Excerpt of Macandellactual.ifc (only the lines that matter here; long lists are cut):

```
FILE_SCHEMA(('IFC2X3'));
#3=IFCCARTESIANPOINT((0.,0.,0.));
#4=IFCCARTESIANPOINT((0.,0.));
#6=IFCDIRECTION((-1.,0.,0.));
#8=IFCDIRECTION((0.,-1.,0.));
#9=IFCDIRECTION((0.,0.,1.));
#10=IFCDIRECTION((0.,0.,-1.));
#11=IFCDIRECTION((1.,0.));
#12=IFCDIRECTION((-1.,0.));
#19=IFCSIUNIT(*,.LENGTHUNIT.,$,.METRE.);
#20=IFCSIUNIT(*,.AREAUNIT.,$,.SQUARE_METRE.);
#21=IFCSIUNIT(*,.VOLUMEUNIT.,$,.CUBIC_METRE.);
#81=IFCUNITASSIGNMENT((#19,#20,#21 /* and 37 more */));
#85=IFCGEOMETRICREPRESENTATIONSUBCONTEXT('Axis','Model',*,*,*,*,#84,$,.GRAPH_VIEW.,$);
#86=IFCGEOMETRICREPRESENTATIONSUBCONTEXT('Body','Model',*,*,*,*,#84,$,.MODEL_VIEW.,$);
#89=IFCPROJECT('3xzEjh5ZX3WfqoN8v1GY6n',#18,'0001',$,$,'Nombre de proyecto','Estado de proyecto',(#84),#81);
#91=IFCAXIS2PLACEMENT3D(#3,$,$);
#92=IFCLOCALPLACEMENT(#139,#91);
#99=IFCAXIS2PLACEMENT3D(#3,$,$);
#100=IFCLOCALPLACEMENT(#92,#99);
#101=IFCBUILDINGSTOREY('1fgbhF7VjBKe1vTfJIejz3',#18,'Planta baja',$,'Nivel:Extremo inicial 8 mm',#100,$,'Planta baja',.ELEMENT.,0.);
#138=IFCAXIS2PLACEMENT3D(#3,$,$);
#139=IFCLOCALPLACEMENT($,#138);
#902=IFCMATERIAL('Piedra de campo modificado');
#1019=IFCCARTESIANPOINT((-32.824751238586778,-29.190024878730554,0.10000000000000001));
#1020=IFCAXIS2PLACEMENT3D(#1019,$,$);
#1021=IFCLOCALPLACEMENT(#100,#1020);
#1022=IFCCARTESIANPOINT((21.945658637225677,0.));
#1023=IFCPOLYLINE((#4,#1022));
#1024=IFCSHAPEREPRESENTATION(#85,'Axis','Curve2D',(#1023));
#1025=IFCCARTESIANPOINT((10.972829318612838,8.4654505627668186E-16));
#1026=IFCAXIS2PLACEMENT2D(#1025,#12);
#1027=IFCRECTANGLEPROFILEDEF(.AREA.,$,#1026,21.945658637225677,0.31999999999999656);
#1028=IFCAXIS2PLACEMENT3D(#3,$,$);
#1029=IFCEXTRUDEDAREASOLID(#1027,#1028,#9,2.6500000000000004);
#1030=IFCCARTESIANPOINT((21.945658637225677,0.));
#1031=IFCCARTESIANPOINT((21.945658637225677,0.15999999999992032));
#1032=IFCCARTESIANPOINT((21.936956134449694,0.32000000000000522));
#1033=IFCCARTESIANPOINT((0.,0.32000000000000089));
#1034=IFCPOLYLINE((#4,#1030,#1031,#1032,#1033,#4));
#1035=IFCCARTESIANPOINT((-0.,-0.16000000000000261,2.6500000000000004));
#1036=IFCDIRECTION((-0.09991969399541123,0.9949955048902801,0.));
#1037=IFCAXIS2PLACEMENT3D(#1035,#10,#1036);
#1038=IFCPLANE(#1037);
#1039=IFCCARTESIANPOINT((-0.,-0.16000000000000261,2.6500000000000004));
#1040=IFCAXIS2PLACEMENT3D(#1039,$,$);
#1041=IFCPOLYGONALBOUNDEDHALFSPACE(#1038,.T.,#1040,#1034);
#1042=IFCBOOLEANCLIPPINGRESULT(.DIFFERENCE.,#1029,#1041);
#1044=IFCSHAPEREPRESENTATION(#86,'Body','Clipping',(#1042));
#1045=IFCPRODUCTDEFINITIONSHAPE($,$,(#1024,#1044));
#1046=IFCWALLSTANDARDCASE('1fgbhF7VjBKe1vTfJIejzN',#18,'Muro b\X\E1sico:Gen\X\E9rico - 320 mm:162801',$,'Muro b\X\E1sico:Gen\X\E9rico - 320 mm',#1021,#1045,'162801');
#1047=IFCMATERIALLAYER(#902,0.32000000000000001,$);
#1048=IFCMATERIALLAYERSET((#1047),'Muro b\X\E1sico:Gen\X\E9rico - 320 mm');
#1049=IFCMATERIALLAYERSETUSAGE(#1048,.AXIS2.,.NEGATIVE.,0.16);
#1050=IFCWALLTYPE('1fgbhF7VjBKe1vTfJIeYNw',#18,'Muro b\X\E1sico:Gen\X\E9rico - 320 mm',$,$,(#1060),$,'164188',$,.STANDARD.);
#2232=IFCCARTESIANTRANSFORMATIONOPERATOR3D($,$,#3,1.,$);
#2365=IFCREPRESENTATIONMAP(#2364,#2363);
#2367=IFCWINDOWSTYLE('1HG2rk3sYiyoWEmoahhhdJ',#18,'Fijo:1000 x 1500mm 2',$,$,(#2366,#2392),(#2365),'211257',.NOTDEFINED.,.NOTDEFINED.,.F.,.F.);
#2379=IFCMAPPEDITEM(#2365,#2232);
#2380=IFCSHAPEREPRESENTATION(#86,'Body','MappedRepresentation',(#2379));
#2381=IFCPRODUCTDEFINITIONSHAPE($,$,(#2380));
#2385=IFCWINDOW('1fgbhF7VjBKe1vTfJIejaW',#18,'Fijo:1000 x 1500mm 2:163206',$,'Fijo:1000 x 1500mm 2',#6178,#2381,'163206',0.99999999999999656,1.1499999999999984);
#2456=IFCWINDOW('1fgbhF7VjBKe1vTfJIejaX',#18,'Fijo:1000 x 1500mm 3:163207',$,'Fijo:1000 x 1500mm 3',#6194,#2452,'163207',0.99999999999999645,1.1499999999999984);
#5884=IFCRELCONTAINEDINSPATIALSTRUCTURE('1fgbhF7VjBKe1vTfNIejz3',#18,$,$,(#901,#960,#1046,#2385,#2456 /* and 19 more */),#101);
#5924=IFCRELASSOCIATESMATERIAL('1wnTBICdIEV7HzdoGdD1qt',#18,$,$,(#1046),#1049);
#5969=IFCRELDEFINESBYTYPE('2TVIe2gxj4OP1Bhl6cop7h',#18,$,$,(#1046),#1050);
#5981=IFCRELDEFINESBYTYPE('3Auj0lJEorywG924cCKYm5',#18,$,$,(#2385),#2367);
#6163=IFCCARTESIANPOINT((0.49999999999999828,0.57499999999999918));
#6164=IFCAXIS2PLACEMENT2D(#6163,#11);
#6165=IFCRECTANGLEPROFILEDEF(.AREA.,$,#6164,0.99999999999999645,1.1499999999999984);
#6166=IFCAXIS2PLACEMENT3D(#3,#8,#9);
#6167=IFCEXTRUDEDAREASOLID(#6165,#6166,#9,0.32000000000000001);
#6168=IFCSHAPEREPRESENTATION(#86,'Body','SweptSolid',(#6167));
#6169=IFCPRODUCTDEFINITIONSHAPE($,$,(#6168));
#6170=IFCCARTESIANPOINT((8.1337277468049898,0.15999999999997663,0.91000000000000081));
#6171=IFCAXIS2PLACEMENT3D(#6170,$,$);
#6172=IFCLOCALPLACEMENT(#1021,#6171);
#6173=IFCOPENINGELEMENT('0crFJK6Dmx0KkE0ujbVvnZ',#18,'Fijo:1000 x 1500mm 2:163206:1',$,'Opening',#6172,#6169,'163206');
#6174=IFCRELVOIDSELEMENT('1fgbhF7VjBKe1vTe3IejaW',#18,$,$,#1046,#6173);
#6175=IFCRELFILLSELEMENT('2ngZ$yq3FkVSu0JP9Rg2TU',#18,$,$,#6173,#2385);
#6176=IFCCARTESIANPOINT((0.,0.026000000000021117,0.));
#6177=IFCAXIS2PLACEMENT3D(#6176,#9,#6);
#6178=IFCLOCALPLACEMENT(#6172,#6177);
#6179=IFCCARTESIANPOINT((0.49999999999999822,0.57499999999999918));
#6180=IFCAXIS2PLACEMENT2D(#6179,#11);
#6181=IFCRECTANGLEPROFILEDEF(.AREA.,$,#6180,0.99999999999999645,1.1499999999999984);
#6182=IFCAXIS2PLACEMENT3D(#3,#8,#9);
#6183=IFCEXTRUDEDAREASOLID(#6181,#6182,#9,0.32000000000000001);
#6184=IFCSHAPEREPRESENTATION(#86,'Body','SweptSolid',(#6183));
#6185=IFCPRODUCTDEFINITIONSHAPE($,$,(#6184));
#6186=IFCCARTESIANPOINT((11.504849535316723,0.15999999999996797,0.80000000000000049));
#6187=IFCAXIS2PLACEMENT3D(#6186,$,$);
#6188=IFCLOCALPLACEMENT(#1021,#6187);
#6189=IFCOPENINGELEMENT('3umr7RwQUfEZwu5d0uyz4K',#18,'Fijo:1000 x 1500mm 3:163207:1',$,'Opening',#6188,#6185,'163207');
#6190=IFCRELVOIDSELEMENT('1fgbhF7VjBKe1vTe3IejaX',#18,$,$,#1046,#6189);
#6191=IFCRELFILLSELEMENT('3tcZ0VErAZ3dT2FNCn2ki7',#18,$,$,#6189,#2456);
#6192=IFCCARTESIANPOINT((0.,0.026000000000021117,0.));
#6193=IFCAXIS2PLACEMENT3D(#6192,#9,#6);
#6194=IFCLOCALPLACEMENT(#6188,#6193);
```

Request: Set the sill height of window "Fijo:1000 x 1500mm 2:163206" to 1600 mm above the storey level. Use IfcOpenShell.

```python
import numpy as np
import ifcopenshell
import ifcopenshell.api.geometry
import ifcopenshell.geom
import ifcopenshell.util.element
import ifcopenshell.util.placement
import ifcopenshell.util.shape
import ifcopenshell.util.unit

model = ifcopenshell.open("Macandellactual.ifc")
unit_scale = ifcopenshell.util.unit.calculate_unit_scale(model)

window = model.by_id(2385)
opening = window.FillsVoids[0].RelatingOpeningElement
storey = ifcopenshell.util.element.get_container(window, ifc_class="IfcBuildingStorey")
level = ifcopenshell.util.placement.get_local_placement(storey.ObjectPlacement)[2, 3]

# The opening's origin need not be at the sill, so measure its lowest point.
shape = ifcopenshell.geom.create_shape(ifcopenshell.geom.settings(), opening)
bottom = ifcopenshell.util.shape.get_shape_bottom_elevation(shape, shape.geometry) / unit_scale
dz = level + 1.6 / unit_scale - bottom

shift = np.array([0.0, 0.0, dz])
# The window is placed relative to its opening, so it follows when the opening moves.
matrix = ifcopenshell.util.placement.get_local_placement(opening.ObjectPlacement)
matrix[:3, 3] += shift
ifcopenshell.api.geometry.edit_object_placement(
    model, product=opening, matrix=matrix, is_si=False, should_transform_children=True
)

print(f"moved by {dz * unit_scale:+.3f} m")

model.write("Macandellactual_v2.ifc")
```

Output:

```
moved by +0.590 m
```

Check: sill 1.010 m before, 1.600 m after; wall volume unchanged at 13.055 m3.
